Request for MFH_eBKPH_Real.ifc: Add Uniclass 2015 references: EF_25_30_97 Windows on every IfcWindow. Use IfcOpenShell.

First a look at what the model holds.

```python
import ifcopenshell

model = ifcopenshell.open("MFH_eBKPH_Real.ifc")
print(model.schema)
print("classifications:", [c.Name for c in model.by_type("IfcClassification")])
for ifc_class in ("IfcDoor", "IfcRoof", "IfcStair", "IfcWall", "IfcWindow"):
    print(ifc_class, len(model.by_type(ifc_class)))
```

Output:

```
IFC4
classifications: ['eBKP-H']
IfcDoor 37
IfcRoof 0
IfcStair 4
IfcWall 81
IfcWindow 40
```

```python
import ifcopenshell
import ifcopenshell.api.classification

model = ifcopenshell.open("MFH_eBKPH_Real.ifc")

system = ifcopenshell.api.classification.add_classification(model, classification="Uniclass 2015")

codes = {
    "IfcWindow": ("EF_25_30_97", "Windows"),
}
for ifc_class, (code, name) in codes.items():
    products = model.by_type(ifc_class)
    ifcopenshell.api.classification.add_reference(
        model, products=products, classification=system, identification=code, name=name
    )
    print(code, len(products))

model.write("MFH_eBKPH_Real_updated.ifc")
```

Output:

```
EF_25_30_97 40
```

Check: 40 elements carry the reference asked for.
